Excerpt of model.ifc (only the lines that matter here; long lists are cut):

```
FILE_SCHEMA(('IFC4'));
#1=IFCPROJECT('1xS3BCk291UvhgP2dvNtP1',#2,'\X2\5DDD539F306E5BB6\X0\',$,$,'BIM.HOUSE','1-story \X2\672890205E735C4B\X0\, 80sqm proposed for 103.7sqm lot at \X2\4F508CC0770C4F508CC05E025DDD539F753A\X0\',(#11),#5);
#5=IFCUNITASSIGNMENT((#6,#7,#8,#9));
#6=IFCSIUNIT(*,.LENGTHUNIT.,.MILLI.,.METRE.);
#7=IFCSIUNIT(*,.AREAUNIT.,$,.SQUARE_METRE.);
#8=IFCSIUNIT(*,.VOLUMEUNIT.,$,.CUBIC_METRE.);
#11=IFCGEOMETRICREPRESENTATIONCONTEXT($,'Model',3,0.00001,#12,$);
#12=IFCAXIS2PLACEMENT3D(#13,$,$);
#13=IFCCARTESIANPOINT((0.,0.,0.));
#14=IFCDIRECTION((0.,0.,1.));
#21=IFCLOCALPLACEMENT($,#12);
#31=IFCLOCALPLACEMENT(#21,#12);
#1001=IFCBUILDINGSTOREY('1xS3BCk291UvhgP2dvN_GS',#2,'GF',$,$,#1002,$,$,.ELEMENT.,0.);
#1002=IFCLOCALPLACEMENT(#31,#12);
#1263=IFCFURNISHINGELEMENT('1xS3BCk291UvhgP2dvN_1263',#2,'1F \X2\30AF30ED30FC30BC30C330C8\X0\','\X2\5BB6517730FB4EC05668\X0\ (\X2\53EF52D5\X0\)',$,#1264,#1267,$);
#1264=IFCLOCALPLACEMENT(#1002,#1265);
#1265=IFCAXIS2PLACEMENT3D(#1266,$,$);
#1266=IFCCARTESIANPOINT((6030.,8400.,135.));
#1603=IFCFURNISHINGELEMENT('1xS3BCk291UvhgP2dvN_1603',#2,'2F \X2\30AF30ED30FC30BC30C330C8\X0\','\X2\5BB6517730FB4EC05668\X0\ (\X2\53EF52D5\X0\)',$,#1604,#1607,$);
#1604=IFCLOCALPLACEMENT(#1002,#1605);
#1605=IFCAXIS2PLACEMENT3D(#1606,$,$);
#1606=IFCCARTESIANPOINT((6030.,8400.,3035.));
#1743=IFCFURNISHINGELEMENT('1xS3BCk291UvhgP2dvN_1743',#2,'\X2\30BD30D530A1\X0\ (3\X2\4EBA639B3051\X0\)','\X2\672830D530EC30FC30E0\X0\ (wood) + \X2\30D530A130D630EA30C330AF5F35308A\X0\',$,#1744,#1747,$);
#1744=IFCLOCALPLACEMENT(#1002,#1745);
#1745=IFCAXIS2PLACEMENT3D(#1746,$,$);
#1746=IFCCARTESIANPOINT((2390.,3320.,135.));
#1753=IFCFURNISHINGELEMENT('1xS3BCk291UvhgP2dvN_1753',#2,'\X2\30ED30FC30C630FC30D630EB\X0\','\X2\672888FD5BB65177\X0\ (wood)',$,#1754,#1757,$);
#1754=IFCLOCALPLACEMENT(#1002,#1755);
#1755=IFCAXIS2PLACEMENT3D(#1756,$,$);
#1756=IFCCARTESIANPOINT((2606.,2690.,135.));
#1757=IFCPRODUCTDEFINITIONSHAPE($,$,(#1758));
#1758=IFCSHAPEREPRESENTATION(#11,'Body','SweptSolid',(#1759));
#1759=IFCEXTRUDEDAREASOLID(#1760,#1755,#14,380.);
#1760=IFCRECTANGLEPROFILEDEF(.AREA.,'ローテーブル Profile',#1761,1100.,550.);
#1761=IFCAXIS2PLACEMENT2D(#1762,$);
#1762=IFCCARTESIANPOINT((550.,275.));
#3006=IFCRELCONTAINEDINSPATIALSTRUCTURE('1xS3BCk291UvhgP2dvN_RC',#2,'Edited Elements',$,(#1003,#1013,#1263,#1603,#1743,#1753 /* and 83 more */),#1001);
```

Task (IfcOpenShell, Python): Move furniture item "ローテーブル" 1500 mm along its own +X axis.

```python
import ifcopenshell
import ifcopenshell.api.geometry
import ifcopenshell.util.placement
import ifcopenshell.util.unit

model = ifcopenshell.open("model.ifc")
unit_scale = ifcopenshell.util.unit.calculate_unit_scale(model)

item = model.by_guid("1xS3BCk291UvhgP2dvN_1753")
matrix = ifcopenshell.util.placement.get_local_placement(item.ObjectPlacement)
matrix[:3, 3] += matrix[:3, 0] * 1.5 / unit_scale
ifcopenshell.api.geometry.edit_object_placement(model, product=item, matrix=matrix, is_si=False)

print(ifcopenshell.util.placement.get_local_placement(item.ObjectPlacement).round(3) + 0.0)

model.write("model_rev.ifc")
```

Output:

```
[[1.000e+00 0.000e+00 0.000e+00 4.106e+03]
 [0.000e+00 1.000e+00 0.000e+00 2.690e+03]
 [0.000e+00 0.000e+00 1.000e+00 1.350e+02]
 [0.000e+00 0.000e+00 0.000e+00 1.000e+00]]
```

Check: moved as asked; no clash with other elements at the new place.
